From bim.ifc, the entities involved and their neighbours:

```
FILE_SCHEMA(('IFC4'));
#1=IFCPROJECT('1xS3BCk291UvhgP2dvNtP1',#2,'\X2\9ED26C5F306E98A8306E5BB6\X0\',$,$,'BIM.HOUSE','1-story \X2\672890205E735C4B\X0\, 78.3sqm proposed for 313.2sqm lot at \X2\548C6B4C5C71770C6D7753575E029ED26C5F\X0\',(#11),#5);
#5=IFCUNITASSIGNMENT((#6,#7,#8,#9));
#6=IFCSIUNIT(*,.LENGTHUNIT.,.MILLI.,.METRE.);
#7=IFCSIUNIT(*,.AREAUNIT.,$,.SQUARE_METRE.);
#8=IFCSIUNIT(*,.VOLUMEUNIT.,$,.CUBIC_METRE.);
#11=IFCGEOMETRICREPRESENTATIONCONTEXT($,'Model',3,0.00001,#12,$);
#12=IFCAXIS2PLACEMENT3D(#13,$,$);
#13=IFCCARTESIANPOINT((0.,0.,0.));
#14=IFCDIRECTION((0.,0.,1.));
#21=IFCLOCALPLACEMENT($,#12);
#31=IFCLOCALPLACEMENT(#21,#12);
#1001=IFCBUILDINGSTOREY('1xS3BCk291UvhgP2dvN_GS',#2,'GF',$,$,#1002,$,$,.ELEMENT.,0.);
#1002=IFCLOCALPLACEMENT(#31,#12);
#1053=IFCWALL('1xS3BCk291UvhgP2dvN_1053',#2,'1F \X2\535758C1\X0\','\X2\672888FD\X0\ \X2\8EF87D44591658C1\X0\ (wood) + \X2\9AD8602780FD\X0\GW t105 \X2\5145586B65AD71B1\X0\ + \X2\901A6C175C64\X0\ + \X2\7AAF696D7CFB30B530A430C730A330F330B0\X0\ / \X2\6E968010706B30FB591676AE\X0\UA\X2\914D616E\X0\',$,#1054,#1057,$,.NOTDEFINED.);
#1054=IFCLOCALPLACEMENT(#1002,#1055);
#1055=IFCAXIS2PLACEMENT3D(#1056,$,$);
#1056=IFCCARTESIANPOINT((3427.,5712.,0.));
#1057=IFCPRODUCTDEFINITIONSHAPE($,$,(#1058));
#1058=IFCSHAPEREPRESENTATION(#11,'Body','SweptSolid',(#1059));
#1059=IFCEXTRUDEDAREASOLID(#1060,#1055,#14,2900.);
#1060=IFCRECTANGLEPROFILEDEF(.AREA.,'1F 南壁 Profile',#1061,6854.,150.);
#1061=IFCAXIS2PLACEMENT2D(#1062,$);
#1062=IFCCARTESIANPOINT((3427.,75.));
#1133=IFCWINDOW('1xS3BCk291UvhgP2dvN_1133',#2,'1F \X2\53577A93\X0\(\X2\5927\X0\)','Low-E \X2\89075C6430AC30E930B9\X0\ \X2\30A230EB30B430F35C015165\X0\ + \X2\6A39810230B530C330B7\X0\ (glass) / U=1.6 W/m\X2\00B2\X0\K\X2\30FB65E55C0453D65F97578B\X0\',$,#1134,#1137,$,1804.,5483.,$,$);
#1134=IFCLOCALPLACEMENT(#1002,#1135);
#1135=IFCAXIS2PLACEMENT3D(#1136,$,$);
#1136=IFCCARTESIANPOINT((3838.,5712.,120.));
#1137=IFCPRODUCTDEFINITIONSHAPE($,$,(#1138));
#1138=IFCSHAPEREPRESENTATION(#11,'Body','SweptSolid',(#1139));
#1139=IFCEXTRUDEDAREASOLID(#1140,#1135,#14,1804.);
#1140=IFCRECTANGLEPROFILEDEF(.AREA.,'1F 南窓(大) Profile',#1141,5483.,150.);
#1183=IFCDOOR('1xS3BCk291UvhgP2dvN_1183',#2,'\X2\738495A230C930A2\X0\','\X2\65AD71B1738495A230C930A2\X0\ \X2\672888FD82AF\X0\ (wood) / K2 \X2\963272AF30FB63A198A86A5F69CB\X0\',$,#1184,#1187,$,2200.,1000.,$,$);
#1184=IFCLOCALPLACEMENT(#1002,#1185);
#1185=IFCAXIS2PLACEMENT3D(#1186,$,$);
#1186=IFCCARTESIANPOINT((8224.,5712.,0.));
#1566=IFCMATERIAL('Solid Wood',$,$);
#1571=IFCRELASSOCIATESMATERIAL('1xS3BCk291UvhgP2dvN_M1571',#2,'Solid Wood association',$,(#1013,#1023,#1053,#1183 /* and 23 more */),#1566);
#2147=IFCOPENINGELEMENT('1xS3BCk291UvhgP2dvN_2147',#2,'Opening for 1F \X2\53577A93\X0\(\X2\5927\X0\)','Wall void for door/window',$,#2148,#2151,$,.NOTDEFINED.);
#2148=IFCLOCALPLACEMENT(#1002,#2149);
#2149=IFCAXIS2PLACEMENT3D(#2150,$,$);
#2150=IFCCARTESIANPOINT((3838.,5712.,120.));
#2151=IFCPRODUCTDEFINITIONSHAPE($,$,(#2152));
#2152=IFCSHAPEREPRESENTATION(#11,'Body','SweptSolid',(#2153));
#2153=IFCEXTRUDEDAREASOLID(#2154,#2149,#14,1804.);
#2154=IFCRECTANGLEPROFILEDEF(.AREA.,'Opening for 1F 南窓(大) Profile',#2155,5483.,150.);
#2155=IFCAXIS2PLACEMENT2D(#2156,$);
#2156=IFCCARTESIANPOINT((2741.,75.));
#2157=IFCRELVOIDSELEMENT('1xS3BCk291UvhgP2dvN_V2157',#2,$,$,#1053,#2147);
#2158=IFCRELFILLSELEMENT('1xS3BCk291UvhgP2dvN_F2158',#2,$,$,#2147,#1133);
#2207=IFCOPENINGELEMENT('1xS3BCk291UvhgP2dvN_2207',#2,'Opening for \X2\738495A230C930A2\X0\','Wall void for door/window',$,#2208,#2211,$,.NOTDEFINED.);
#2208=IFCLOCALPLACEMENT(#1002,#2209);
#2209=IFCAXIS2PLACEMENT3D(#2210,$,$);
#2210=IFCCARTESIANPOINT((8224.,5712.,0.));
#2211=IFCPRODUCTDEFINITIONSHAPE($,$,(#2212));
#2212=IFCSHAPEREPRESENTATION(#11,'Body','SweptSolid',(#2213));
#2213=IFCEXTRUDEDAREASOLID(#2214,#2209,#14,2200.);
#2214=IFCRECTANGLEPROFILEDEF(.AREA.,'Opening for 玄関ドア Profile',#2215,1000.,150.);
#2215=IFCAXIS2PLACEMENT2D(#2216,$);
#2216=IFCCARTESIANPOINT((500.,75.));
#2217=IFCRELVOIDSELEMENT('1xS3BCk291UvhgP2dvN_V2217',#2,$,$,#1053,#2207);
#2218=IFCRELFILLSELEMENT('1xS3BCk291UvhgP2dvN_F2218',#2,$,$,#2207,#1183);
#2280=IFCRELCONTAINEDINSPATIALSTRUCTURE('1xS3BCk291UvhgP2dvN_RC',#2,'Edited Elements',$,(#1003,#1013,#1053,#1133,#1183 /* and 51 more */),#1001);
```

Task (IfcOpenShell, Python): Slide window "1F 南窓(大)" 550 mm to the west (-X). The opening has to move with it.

```python
import ifcopenshell
import ifcopenshell.api.geometry
import ifcopenshell.util.placement
import ifcopenshell.util.unit

model = ifcopenshell.open("bim.ifc")
unit_scale = ifcopenshell.util.unit.calculate_unit_scale(model)

window = model.by_guid("1xS3BCk291UvhgP2dvN_1133")
opening = window.FillsVoids[0].RelatingOpeningElement
wall = opening.VoidsElements[0].RelatingBuildingElement

wall_matrix = ifcopenshell.util.placement.get_local_placement(wall.ObjectPlacement)
shift = wall_matrix[:3, 0] * -0.55 / unit_scale
before = ifcopenshell.util.placement.get_local_placement(window.ObjectPlacement)[:3, 3].copy()

# The window is not placed relative to its opening, so move both.
for product in (opening, window):
    matrix = ifcopenshell.util.placement.get_local_placement(product.ObjectPlacement)
    matrix[:3, 3] += shift
    ifcopenshell.api.geometry.edit_object_placement(model, product=product, matrix=matrix, is_si=False)

after = ifcopenshell.util.placement.get_local_placement(window.ObjectPlacement)[:3, 3]
print("window moved by", (after - before).round(3) + 0.0)

model.write("bim_v2.ifc")
```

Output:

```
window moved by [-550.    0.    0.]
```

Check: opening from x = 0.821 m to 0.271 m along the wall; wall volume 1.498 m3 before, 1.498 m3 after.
